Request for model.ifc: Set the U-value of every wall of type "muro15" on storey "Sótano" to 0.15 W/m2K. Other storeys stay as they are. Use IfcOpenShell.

First a look at what the model holds.

```python
import ifcopenshell
import ifcopenshell.util.element

model = ifcopenshell.open("model.ifc")
print(model.schema)
storey = next(s for s in model.by_type("IfcBuildingStorey") if s.Name == "Sótano")
walls = [e for e in ifcopenshell.util.element.get_decomposition(storey) if e.is_a("IfcWall")]
seen = {}
for e in walls:
    element_type = ifcopenshell.util.element.get_type(e)
    key = (element_type.Name if element_type != e and element_type else None, ifcopenshell.util.element.get_pset(e, "Pset_WallCommon", "ThermalTransmittance"))
    seen[key] = seen.get(key, 0) + 1
for (name, value), count in sorted(seen.items(), key=str):
    print(count, "x", name, "|", value)
```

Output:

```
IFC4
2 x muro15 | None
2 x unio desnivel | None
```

```python
import ifcopenshell
import ifcopenshell.api.pset
import ifcopenshell.util.element

model = ifcopenshell.open("model.ifc")

storey = next(s for s in model.by_type("IfcBuildingStorey") if s.Name == "Sótano")
walls = [e for e in ifcopenshell.util.element.get_decomposition(storey) if e.is_a("IfcWall")]

count = 0
for e in walls:
    element_type = ifcopenshell.util.element.get_type(e)
    if element_type in (None, e) or element_type.Name != "muro15":
        continue
    # add_pset returns the element's existing set when there is one.
    pset = ifcopenshell.api.pset.add_pset(model, product=e, name="Pset_WallCommon")
    ifcopenshell.api.pset.edit_pset(model, pset=pset, properties={"ThermalTransmittance": 0.15})
    count += 1

print(count, "walls updated")

model.write("model_updated.ifc")
```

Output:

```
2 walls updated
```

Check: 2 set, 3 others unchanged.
